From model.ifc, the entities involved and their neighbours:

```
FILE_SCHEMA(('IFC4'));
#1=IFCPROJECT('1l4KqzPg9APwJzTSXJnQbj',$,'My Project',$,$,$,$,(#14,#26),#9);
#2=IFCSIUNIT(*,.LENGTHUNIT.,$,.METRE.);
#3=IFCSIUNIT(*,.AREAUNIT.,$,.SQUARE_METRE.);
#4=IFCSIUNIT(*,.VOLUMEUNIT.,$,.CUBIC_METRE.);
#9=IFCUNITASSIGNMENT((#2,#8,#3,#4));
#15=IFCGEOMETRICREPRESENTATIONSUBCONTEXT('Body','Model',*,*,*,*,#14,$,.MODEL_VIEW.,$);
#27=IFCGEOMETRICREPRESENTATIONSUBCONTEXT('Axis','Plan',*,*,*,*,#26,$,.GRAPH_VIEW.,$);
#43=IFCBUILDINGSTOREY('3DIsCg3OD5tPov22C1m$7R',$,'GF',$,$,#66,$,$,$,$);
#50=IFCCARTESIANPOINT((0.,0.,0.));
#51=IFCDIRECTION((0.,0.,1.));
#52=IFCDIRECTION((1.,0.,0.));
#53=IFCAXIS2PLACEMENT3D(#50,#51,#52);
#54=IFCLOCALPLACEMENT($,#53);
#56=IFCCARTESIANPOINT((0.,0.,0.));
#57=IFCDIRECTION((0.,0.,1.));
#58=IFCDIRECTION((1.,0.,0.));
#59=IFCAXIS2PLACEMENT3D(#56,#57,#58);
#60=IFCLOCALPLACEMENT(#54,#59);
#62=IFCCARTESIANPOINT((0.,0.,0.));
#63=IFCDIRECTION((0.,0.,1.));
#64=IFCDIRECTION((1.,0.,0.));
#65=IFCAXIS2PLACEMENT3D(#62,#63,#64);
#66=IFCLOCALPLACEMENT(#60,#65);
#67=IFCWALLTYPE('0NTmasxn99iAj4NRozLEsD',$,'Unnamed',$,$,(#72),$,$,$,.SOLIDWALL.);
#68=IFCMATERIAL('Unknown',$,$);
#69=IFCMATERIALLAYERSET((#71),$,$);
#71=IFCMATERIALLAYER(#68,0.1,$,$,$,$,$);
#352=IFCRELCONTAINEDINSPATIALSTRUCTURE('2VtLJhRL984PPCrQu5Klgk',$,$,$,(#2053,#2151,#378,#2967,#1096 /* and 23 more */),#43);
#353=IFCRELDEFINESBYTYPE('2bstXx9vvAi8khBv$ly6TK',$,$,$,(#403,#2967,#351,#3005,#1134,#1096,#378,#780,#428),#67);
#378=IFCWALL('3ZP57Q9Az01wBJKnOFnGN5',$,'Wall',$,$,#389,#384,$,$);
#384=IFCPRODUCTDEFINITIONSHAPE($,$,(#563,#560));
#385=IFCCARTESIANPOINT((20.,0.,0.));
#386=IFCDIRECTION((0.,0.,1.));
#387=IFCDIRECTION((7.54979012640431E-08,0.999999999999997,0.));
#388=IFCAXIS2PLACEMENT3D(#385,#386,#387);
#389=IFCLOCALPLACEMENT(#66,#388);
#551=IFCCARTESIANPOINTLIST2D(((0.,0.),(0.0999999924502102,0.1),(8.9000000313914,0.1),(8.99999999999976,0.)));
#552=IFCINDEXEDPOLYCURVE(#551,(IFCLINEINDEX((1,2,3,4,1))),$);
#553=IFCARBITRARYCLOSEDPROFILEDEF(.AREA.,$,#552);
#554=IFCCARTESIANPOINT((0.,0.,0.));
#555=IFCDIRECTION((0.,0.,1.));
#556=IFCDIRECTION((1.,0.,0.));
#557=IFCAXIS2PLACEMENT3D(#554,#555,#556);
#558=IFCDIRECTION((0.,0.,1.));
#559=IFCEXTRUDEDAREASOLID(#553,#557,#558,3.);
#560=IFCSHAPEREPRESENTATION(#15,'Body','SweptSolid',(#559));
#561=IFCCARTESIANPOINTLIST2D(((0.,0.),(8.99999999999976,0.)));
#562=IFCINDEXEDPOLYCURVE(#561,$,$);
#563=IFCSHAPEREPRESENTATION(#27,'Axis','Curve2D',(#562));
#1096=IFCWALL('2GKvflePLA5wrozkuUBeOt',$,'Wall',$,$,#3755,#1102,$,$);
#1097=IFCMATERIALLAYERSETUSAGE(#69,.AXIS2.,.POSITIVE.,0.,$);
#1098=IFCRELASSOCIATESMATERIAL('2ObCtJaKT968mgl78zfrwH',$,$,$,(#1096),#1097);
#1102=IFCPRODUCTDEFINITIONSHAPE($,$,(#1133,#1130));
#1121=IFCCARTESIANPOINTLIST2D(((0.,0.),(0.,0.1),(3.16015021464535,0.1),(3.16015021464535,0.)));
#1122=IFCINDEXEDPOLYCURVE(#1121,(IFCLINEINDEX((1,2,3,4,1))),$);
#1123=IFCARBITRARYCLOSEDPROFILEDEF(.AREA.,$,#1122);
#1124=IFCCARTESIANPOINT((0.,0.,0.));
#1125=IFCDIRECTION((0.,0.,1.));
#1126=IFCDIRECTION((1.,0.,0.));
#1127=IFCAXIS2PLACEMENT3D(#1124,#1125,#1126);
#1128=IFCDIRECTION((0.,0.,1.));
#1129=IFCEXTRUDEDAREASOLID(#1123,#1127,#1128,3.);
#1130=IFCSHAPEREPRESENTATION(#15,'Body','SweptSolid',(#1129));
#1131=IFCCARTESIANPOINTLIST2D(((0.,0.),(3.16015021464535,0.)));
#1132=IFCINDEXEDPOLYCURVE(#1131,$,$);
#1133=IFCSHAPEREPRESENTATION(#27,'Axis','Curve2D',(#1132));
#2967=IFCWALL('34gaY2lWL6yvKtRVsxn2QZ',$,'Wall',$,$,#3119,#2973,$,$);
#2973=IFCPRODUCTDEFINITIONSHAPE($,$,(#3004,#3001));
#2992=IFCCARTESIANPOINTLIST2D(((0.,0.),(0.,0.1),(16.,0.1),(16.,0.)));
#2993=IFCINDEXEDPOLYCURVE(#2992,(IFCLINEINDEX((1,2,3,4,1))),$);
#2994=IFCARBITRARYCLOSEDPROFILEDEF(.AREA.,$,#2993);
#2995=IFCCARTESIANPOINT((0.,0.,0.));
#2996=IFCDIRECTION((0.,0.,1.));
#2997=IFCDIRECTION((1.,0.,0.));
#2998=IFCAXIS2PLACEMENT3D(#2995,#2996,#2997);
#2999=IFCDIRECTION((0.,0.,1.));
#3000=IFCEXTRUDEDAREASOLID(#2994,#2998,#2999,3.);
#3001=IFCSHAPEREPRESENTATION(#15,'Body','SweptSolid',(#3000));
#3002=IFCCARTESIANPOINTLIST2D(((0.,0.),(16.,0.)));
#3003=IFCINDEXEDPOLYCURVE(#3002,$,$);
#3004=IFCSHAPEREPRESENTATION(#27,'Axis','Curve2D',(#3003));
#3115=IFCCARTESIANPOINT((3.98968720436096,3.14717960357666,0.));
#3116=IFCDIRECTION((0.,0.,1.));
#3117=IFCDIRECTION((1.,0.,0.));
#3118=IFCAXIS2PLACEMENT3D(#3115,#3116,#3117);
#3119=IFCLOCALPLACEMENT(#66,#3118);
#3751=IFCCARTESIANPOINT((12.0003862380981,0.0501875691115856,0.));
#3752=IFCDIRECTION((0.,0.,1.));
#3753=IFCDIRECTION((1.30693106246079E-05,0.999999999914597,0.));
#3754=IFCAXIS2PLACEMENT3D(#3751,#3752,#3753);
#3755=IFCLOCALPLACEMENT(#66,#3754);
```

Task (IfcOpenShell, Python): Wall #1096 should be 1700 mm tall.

```python
import ifcopenshell
import ifcopenshell.geom
import ifcopenshell.util.representation
import ifcopenshell.util.shape
import ifcopenshell.util.unit

model = ifcopenshell.open("model.ifc")
unit_scale = ifcopenshell.util.unit.calculate_unit_scale(model)
settings = ifcopenshell.geom.settings()


def volume(element):
    """Net volume in cubic metres, openings subtracted."""
    shape = ifcopenshell.geom.create_shape(settings, element)
    return ifcopenshell.util.shape.get_volume(shape.geometry)


wall = model.by_guid("2GKvflePLA5wrozkuUBeOt")
before = volume(wall)

body = ifcopenshell.util.representation.get_representation(wall, "Model", "Body")
solid = body.Items[0]
old_height = solid.Depth
solid.Depth = 1.7 / unit_scale
after = volume(wall)

print(f"height {old_height:g} -> {solid.Depth:g}, volume {before:.3f} -> {after:.3f} m3")

model.write("model-out.ifc")
```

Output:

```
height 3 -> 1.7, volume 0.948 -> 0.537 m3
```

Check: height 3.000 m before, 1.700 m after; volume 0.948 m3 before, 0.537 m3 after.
